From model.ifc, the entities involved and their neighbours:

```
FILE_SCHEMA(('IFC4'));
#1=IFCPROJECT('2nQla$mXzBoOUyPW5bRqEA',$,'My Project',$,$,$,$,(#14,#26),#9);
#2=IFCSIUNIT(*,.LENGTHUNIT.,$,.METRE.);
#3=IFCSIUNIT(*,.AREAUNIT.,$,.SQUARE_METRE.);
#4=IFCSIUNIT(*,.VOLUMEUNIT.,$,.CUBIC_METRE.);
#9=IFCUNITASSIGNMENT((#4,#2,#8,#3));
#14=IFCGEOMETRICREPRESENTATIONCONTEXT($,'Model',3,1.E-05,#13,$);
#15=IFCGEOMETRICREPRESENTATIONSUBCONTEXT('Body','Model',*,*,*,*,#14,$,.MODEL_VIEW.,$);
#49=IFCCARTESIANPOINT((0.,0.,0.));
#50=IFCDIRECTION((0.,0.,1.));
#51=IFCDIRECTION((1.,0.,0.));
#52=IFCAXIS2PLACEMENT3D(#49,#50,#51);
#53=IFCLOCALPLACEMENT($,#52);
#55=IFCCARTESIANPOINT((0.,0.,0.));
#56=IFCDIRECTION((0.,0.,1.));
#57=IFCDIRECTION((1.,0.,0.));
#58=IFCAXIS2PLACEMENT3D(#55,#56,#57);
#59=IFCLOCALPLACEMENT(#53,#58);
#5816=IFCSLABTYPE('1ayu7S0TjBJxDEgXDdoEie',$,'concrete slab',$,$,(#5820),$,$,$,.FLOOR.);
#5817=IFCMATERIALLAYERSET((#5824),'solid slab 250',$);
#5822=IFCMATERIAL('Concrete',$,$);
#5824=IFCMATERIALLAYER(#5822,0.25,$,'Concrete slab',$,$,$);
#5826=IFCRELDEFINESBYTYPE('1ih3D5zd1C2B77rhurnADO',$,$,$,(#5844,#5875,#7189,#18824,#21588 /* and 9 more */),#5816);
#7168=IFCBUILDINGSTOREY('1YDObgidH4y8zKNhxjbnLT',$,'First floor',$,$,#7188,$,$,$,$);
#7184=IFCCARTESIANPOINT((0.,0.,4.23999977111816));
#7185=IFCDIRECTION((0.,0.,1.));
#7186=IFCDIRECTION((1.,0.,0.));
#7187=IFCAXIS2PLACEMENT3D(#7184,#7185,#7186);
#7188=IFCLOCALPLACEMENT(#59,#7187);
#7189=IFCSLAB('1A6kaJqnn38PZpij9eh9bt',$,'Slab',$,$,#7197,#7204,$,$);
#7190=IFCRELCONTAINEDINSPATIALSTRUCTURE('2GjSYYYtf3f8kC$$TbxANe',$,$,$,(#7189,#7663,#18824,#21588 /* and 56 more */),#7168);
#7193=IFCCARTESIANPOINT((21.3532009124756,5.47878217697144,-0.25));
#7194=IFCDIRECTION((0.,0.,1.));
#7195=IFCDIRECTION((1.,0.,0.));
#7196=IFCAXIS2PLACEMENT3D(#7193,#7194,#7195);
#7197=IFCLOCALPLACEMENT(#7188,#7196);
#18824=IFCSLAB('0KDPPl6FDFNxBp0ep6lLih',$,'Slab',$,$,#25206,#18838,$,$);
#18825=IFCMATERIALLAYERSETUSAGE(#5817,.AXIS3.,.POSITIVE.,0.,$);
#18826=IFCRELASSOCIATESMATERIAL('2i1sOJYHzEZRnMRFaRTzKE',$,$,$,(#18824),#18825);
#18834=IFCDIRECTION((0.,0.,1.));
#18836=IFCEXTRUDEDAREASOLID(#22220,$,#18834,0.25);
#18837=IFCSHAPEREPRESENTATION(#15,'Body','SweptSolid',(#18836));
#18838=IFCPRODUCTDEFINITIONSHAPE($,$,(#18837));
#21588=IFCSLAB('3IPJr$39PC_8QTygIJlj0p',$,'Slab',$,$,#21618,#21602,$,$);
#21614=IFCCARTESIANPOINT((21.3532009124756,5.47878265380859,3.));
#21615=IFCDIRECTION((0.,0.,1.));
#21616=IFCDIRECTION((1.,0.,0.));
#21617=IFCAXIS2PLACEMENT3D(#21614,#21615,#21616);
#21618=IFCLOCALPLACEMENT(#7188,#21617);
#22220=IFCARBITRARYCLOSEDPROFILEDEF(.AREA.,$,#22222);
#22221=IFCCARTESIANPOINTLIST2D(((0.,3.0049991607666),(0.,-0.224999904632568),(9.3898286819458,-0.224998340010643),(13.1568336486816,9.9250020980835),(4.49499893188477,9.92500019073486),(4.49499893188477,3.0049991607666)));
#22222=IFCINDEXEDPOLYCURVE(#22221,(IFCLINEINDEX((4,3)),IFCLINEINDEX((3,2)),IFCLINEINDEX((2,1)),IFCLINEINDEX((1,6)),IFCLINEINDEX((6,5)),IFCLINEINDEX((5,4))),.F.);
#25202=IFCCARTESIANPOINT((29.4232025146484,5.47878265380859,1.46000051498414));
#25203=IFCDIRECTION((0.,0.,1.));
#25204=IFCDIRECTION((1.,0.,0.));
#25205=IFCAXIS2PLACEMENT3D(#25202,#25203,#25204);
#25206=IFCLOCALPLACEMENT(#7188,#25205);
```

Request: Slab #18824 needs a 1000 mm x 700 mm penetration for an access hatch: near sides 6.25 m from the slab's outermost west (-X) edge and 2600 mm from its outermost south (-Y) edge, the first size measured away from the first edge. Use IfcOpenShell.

```python
import numpy as np
import ifcopenshell
import ifcopenshell.api.feature
import ifcopenshell.api.geometry
import ifcopenshell.api.root
import ifcopenshell.geom
import ifcopenshell.util.placement
import ifcopenshell.util.representation
import ifcopenshell.util.shape
import ifcopenshell.util.unit

model = ifcopenshell.open("model.ifc")
unit_scale = ifcopenshell.util.unit.calculate_unit_scale(model)
settings = ifcopenshell.geom.settings()


def volume(element):
    """Net volume in cubic metres, openings subtracted."""
    shape = ifcopenshell.geom.create_shape(settings, element)
    return ifcopenshell.util.shape.get_volume(shape.geometry)


slab = model.by_guid("0KDPPl6FDFNxBp0ep6lLih")
before = volume(slab)

# Extent in the slab's own axes, in metres. The edges named are its -X and -Y sides.
slab_shape = ifcopenshell.geom.create_shape(settings, slab)
vertices = ifcopenshell.util.shape.get_vertices(slab_shape.geometry)
x_min, y_min, bottom = vertices.min(axis=0)
top = vertices[:, 2].max()

opening = ifcopenshell.api.root.create_entity(model, ifc_class="IfcOpeningElement", name="Access hatch opening", predefined_type="OPENING")
context = ifcopenshell.util.representation.get_context(model, "Model", "Body", "MODEL_VIEW")
width, depth = 1, 0.7
outline = [(0.0, 0.0), (width, 0.0), (width, depth), (0.0, depth), (0.0, 0.0)]
# Overshoot both faces by 50 mm so the cut is clean.
shape = ifcopenshell.api.geometry.add_slab_representation(
    model, context=context, depth=top - bottom + 0.1, polyline=outline
)
ifcopenshell.api.geometry.assign_representation(model, product=opening, representation=shape)

matrix = ifcopenshell.util.placement.get_local_placement(slab.ObjectPlacement)
matrix[:, 3] = matrix @ np.append(np.array([x_min + 6.25, y_min + 2.6, bottom - 0.05]) / unit_scale, 1.0)
ifcopenshell.api.geometry.edit_object_placement(model, product=opening, matrix=matrix, is_si=False)
ifcopenshell.api.feature.add_feature(model, feature=opening, element=slab)

after = volume(slab)

print(f"slab volume {before:.3f} -> {after:.3f} m3")

model.write("model_edited.ifc")
```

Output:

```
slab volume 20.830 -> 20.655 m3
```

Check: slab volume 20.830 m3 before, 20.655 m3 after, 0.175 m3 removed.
